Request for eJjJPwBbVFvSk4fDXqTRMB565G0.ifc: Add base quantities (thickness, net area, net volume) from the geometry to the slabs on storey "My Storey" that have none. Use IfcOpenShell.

First a look at what the model holds.

```python
import ifcopenshell
import ifcopenshell.util.element
import ifcopenshell.util.unit

model = ifcopenshell.open("eJjJPwBbVFvSk4fDXqTRMB565G0.ifc")
print(model.schema)
for unit_type in ("LENGTHUNIT", "AREAUNIT", "VOLUMEUNIT"):
    print(unit_type, ifcopenshell.util.unit.calculate_unit_scale(model, unit_type))
storey = next(s for s in model.by_type("IfcBuildingStorey") if s.Name == "My Storey")
slabs = [e for e in ifcopenshell.util.element.get_decomposition(storey) if e.is_a("IfcSlab")]
for e in sorted(slabs, key=lambda e: e.id()):
    print(e.id(), e.is_a(), e.Name, list(ifcopenshell.util.element.get_psets(e, qtos_only=True)), sep=" | ")
```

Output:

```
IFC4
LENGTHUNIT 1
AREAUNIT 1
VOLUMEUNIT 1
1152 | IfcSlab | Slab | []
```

```python
import ifcopenshell
import ifcopenshell.api.pset
import ifcopenshell.geom
import ifcopenshell.util.element
import ifcopenshell.util.shape
import ifcopenshell.util.unit

model = ifcopenshell.open("eJjJPwBbVFvSk4fDXqTRMB565G0.ifc")
unit_scale = ifcopenshell.util.unit.calculate_unit_scale(model)
area_scale = ifcopenshell.util.unit.calculate_unit_scale(model, "AREAUNIT")
volume_scale = ifcopenshell.util.unit.calculate_unit_scale(model, "VOLUMEUNIT")
settings = ifcopenshell.geom.settings()

storey = next(s for s in model.by_type("IfcBuildingStorey") if s.Name == "My Storey")
slabs = [e for e in ifcopenshell.util.element.get_decomposition(storey) if e.is_a("IfcSlab")]

for e in sorted(slabs, key=lambda e: e.id()):
    if ifcopenshell.util.element.get_psets(e, qtos_only=True, should_inherit=False):
        continue
    # Geometry comes back in metres, in the element's own axes.
    shape = ifcopenshell.geom.create_shape(settings, e)
    values = {
        "Width": ifcopenshell.util.shape.get_z(shape.geometry) / unit_scale,
        "NetArea": ifcopenshell.util.shape.get_footprint_area(shape.geometry) / area_scale,
        "NetVolume": ifcopenshell.util.shape.get_volume(shape.geometry) / volume_scale,
    }
    qto = ifcopenshell.api.pset.add_qto(model, product=e, name="Qto_SlabBaseQuantities")
    ifcopenshell.api.pset.edit_qto(model, qto=qto, properties=values)
    print(e.id(), {k: round(v, 3) for k, v in values.items()})

model.write("eJjJPwBbVFvSk4fDXqTRMB565G0-out.ifc")
```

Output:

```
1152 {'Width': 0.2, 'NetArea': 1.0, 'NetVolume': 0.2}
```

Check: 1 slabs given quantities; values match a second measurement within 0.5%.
